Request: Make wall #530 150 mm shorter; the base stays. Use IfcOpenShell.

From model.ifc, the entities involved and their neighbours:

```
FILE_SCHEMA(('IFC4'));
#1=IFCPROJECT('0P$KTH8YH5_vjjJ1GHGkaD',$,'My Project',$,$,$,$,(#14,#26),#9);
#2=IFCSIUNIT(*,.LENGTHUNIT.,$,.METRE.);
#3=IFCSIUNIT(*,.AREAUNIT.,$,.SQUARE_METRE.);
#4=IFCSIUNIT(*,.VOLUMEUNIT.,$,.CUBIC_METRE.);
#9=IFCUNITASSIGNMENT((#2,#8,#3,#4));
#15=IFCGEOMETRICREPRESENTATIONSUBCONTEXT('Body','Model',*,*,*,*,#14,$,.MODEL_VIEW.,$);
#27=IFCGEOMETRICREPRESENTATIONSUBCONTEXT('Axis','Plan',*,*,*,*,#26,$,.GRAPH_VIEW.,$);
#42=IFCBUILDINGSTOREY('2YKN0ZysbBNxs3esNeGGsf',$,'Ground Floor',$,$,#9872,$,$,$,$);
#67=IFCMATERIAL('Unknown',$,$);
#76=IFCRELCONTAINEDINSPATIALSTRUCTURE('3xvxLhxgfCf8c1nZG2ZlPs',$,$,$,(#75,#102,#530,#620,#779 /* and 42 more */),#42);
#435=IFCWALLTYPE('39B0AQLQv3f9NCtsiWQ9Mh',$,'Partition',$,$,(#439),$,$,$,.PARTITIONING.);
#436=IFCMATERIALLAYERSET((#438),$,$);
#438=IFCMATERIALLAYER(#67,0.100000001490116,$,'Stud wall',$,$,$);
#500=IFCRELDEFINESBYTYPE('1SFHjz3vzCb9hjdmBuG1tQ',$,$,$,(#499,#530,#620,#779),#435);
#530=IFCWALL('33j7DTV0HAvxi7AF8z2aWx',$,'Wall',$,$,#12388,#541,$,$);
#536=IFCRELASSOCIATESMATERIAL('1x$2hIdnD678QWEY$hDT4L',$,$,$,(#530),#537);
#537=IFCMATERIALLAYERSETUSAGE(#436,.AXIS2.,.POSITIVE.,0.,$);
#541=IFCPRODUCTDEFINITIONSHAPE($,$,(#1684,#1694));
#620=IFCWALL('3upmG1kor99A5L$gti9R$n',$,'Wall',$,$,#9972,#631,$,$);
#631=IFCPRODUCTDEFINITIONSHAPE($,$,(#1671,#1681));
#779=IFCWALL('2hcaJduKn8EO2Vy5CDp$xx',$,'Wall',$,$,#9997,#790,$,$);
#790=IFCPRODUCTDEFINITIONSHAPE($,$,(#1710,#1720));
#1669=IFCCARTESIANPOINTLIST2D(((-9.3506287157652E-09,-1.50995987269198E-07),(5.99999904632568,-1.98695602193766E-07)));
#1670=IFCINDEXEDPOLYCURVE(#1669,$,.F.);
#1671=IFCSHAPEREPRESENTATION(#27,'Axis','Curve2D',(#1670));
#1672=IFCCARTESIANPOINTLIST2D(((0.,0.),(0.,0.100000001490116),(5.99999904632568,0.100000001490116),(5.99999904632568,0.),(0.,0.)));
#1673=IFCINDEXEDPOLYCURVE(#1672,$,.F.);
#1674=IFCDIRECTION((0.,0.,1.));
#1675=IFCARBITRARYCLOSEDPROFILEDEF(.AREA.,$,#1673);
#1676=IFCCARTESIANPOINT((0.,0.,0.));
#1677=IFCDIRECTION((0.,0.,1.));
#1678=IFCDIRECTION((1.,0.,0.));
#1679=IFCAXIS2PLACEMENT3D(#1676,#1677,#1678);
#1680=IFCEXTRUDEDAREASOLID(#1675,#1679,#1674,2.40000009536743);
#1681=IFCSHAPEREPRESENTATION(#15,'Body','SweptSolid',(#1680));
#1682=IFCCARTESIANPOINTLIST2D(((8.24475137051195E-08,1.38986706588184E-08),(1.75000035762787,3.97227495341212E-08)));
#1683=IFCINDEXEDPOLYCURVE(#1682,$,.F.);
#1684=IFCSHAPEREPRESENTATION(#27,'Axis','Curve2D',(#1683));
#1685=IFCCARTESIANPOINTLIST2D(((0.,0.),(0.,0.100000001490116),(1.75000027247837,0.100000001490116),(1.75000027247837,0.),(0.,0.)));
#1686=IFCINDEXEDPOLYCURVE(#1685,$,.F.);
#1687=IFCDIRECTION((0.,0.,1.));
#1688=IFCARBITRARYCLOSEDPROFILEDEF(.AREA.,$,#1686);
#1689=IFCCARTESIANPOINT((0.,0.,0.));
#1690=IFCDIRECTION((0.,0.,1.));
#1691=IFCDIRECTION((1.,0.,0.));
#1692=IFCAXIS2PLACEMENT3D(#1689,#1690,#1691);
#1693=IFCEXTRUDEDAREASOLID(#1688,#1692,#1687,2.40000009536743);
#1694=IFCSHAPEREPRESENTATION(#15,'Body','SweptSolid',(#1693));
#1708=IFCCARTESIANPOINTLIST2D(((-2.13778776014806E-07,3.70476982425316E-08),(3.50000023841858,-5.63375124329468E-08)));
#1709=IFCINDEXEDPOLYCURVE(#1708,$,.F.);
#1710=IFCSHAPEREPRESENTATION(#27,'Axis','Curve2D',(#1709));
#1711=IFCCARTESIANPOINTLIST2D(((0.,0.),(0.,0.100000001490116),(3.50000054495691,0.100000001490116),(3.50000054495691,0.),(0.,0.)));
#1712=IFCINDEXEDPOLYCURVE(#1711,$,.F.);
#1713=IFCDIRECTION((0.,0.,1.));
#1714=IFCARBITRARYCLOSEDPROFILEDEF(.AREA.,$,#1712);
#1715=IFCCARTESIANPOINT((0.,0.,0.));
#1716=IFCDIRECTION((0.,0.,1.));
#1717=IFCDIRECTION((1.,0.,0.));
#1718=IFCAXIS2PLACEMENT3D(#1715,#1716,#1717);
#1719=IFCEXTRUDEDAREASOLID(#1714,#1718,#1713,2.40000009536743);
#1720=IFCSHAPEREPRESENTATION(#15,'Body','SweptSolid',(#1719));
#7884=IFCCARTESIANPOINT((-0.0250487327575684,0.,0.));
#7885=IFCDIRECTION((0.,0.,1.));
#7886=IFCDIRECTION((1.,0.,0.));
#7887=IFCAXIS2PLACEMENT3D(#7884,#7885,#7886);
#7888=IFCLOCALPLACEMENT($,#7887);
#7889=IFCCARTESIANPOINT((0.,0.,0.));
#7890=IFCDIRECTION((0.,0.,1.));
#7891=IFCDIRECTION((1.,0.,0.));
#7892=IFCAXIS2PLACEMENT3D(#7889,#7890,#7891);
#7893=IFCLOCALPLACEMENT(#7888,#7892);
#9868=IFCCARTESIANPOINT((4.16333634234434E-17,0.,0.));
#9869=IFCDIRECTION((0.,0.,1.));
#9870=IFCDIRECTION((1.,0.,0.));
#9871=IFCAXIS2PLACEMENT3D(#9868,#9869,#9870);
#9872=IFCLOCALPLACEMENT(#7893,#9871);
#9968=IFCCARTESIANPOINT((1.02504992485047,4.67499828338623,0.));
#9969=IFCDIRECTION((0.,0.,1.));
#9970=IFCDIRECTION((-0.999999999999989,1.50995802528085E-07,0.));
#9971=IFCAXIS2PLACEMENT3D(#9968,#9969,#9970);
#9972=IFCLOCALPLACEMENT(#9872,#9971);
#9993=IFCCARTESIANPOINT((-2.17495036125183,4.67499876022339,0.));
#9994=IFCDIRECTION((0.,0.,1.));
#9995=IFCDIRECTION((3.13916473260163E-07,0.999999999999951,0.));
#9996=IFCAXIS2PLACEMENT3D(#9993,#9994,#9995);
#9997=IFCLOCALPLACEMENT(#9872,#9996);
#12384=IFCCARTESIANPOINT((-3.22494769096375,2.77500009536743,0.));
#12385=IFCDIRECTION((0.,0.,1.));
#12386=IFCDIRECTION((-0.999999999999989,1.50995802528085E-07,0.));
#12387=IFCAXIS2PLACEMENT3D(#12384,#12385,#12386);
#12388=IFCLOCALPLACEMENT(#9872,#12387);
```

```python
import ifcopenshell
import ifcopenshell.geom
import ifcopenshell.util.representation
import ifcopenshell.util.shape
import ifcopenshell.util.unit

model = ifcopenshell.open("model.ifc")
unit_scale = ifcopenshell.util.unit.calculate_unit_scale(model)
settings = ifcopenshell.geom.settings()


def volume(element):
    """Net volume in cubic metres, openings subtracted."""
    shape = ifcopenshell.geom.create_shape(settings, element)
    return ifcopenshell.util.shape.get_volume(shape.geometry)


wall = model.by_guid("33j7DTV0HAvxi7AF8z2aWx")
before = volume(wall)

body = ifcopenshell.util.representation.get_representation(wall, "Model", "Body")
solid = body.Items[0]
old_height = solid.Depth
solid.Depth -= 0.15 / unit_scale
after = volume(wall)

print(f"height {old_height:g} -> {solid.Depth:g}, volume {before:.3f} -> {after:.3f} m3")

model.write("model_updated.ifc")
```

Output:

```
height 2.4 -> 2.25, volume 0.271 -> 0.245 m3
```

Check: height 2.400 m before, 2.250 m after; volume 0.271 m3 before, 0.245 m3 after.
